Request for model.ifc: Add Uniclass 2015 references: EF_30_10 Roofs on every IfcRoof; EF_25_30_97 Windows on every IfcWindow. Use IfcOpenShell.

First a look at what the model holds.

```python
import ifcopenshell

model = ifcopenshell.open("model.ifc")
print(model.schema)
print("classifications:", [c.Name for c in model.by_type("IfcClassification")])
for ifc_class in ("IfcDoor", "IfcRoof", "IfcStair", "IfcWall", "IfcWindow"):
    print(ifc_class, len(model.by_type(ifc_class)))
```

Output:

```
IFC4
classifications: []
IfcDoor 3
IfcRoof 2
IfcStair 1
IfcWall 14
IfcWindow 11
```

```python
import ifcopenshell
import ifcopenshell.api.classification

model = ifcopenshell.open("model.ifc")

system = ifcopenshell.api.classification.add_classification(model, classification="Uniclass 2015")

codes = {
    "IfcRoof": ("EF_30_10", "Roofs"),
    "IfcWindow": ("EF_25_30_97", "Windows"),
}
for ifc_class, (code, name) in codes.items():
    products = model.by_type(ifc_class)
    ifcopenshell.api.classification.add_reference(
        model, products=products, classification=system, identification=code, name=name
    )
    print(code, len(products))

model.write("model_rev.ifc")
```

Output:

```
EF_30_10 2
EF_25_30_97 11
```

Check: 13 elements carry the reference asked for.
